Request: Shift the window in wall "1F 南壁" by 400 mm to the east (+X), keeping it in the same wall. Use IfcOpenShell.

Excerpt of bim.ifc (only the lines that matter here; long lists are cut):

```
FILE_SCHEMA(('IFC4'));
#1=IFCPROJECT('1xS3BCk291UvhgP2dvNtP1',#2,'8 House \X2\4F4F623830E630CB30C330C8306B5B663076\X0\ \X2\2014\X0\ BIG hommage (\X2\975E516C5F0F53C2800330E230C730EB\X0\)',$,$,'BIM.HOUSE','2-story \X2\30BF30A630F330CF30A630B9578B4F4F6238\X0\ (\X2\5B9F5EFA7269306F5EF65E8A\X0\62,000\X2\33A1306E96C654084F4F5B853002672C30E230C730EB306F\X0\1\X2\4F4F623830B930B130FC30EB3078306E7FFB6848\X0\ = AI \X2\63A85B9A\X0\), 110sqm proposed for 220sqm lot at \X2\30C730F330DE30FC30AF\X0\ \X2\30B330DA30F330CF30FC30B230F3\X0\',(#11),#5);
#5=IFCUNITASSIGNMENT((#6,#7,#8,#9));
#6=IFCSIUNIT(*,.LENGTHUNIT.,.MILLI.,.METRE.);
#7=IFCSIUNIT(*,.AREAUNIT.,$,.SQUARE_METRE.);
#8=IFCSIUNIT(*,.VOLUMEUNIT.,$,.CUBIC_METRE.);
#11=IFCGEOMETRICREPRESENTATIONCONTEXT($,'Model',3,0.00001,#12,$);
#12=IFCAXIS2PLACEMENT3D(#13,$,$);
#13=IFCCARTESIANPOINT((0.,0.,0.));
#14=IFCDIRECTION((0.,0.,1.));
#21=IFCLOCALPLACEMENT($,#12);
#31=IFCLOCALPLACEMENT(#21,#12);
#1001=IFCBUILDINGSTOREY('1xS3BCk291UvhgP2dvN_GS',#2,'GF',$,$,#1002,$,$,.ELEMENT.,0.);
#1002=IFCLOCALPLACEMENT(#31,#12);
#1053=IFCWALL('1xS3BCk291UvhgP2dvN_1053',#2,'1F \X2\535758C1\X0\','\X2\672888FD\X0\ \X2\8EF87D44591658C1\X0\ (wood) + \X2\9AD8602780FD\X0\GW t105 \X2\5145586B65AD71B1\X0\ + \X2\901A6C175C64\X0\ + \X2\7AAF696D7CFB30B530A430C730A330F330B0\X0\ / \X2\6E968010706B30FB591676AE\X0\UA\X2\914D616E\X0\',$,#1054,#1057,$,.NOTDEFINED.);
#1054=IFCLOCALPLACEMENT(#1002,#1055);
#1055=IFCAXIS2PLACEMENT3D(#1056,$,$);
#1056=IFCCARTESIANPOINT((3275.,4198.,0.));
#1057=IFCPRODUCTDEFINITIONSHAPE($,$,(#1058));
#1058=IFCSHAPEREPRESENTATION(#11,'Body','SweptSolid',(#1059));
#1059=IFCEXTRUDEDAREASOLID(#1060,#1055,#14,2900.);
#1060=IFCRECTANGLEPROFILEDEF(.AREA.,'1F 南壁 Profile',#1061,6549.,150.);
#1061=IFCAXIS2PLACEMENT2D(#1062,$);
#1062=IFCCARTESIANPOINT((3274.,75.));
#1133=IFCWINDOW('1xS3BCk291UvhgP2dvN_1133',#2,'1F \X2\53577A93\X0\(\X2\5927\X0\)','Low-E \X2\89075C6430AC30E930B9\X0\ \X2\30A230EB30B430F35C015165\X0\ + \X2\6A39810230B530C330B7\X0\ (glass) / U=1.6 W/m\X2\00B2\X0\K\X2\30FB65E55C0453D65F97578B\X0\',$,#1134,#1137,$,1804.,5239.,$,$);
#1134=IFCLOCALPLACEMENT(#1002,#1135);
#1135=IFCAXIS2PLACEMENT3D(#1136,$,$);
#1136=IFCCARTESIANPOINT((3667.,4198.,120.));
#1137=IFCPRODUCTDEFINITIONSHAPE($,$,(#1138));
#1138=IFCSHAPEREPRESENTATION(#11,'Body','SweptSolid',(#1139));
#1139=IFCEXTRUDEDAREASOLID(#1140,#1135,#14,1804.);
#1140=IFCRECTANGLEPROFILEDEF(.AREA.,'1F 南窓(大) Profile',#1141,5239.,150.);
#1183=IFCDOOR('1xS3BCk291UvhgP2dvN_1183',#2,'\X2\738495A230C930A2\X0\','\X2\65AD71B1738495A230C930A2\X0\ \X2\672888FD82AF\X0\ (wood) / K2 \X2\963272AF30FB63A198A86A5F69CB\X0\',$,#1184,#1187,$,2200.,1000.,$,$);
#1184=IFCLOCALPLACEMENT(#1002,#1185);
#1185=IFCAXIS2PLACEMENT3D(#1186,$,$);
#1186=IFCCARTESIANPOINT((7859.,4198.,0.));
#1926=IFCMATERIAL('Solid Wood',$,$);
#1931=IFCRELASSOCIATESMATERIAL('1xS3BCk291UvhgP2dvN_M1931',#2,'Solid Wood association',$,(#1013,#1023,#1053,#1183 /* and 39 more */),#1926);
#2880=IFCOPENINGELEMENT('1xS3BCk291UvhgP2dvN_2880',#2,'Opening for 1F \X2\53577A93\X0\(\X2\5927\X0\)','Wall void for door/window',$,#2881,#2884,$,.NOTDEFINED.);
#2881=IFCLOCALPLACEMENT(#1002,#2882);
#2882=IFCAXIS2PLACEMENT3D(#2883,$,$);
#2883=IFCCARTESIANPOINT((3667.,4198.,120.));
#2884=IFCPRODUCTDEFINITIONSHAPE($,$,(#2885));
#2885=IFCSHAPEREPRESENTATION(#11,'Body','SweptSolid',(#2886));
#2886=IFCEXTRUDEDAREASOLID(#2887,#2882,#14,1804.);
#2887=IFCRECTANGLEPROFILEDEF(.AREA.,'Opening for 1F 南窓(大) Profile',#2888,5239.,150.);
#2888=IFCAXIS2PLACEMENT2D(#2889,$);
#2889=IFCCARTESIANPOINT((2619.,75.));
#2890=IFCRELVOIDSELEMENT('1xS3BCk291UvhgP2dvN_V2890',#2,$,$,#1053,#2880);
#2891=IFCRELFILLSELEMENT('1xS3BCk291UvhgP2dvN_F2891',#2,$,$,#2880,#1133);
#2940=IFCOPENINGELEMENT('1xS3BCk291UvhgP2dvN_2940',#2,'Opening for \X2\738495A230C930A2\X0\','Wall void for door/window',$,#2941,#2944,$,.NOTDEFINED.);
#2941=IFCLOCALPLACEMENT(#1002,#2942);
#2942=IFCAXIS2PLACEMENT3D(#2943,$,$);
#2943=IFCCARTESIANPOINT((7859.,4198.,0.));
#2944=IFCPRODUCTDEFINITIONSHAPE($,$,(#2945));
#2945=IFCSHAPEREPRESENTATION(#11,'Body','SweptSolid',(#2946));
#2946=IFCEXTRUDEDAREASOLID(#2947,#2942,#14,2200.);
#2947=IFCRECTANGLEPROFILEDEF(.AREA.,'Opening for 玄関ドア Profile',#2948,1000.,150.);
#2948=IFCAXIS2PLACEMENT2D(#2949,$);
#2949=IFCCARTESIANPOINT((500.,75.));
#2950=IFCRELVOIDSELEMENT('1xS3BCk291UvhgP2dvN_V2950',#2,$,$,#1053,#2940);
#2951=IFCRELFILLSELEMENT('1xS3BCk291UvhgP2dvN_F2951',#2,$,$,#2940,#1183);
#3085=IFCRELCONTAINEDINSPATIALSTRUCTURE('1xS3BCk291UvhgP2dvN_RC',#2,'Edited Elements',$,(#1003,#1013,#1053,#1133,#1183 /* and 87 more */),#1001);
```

```python
import ifcopenshell
import ifcopenshell.api.geometry
import ifcopenshell.util.placement
import ifcopenshell.util.unit

model = ifcopenshell.open("bim.ifc")
unit_scale = ifcopenshell.util.unit.calculate_unit_scale(model)

window = model.by_guid("1xS3BCk291UvhgP2dvN_1133")
opening = window.FillsVoids[0].RelatingOpeningElement
wall = opening.VoidsElements[0].RelatingBuildingElement

wall_matrix = ifcopenshell.util.placement.get_local_placement(wall.ObjectPlacement)
shift = wall_matrix[:3, 0] * 0.4 / unit_scale
before = ifcopenshell.util.placement.get_local_placement(window.ObjectPlacement)[:3, 3].copy()

# The window is not placed relative to its opening, so move both.
for product in (opening, window):
    matrix = ifcopenshell.util.placement.get_local_placement(product.ObjectPlacement)
    matrix[:3, 3] += shift
    ifcopenshell.api.geometry.edit_object_placement(model, product=product, matrix=matrix, is_si=False)

after = ifcopenshell.util.placement.get_local_placement(window.ObjectPlacement)[:3, 3]
print("window moved by", (after - before).round(3) + 0.0)

model.write("bim_rev.ifc")
```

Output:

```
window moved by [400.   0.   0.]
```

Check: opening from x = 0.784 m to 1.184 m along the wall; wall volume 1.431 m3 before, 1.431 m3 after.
